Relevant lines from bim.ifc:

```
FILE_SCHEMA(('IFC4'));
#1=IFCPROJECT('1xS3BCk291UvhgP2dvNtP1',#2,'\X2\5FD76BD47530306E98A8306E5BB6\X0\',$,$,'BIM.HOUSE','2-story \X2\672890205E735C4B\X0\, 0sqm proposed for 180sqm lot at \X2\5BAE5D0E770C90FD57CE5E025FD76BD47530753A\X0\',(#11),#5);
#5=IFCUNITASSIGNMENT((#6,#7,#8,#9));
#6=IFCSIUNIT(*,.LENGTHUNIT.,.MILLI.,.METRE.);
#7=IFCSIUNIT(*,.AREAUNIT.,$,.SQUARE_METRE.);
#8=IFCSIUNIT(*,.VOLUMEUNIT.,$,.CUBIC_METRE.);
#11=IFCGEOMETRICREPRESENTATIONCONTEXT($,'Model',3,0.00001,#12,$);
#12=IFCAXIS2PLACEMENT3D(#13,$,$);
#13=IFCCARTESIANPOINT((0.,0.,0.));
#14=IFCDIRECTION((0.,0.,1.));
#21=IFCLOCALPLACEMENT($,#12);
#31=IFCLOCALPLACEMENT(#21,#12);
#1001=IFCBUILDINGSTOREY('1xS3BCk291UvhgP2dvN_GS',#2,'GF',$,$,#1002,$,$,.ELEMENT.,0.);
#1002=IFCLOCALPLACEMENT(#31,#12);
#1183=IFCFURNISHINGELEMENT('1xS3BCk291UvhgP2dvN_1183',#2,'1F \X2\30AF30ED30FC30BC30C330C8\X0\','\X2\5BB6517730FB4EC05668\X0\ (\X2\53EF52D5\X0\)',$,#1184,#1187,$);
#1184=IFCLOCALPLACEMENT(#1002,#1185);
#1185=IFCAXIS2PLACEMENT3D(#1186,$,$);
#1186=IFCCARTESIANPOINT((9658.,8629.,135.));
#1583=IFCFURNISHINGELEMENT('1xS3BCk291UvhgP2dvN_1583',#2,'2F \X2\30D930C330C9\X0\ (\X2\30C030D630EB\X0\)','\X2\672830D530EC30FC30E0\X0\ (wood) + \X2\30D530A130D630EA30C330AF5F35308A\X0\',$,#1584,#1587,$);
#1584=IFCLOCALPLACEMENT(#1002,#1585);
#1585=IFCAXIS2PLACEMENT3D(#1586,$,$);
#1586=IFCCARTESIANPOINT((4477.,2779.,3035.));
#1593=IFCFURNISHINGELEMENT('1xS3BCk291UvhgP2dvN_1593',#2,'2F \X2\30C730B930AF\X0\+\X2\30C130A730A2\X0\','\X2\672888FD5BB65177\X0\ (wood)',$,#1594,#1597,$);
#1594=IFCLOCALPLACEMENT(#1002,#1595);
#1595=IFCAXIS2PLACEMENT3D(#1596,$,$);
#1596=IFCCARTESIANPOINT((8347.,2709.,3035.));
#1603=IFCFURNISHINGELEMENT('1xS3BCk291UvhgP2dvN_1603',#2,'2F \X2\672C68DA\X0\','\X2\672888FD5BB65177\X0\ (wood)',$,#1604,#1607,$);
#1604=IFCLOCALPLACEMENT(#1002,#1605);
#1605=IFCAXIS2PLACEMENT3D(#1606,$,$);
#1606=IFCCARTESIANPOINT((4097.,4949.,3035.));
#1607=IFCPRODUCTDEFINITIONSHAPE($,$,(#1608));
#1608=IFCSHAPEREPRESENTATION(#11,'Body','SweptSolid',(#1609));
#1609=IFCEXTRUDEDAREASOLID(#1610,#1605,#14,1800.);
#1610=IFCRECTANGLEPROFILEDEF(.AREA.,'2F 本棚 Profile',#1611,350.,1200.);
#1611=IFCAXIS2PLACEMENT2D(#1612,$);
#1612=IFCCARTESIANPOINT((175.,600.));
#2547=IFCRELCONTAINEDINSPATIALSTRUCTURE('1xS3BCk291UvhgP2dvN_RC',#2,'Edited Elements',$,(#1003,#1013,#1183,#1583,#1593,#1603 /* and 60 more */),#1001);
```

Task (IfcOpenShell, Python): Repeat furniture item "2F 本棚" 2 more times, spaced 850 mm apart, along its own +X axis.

```python
import ifcopenshell
import ifcopenshell.api.geometry
import ifcopenshell.api.root
import ifcopenshell.util.element
import ifcopenshell.util.placement
import ifcopenshell.util.unit

model = ifcopenshell.open("bim.ifc")
unit_scale = ifcopenshell.util.unit.calculate_unit_scale(model)


def reuse_history(source, copy):
    """copy_class also copies each property set's owner history, people and application; keep the originals."""
    for rel in copy.IsDefinedBy:
        if rel.is_a("IfcRelDefinesByProperties") and (history := rel.RelatingPropertyDefinition.OwnerHistory):
            rel.RelatingPropertyDefinition.OwnerHistory = source.OwnerHistory
            ifcopenshell.util.element.remove_deep2(model, history)


source = model.by_guid("1xS3BCk291UvhgP2dvN_1603")
base = ifcopenshell.util.placement.get_local_placement(source.ObjectPlacement)
step = base[:3, 0] * 0.85 / unit_scale

for i in range(1, 3):
    copy = ifcopenshell.api.root.copy_class(model, product=source)
    copy.Representation = ifcopenshell.util.element.copy_deep(
        model, source.Representation, exclude=["IfcGeometricRepresentationContext", "IfcRepresentationMap"]
    )
    reuse_history(source, copy)
    matrix = base.copy()
    matrix[:3, 3] += i * step
    print("added at", matrix[:3, 3].round(3) + 0.0)
    ifcopenshell.api.geometry.edit_object_placement(model, product=copy, matrix=matrix, is_si=False)

model.write("bim_rev.ifc")
```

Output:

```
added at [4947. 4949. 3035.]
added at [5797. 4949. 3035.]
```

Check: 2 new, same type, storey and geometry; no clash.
